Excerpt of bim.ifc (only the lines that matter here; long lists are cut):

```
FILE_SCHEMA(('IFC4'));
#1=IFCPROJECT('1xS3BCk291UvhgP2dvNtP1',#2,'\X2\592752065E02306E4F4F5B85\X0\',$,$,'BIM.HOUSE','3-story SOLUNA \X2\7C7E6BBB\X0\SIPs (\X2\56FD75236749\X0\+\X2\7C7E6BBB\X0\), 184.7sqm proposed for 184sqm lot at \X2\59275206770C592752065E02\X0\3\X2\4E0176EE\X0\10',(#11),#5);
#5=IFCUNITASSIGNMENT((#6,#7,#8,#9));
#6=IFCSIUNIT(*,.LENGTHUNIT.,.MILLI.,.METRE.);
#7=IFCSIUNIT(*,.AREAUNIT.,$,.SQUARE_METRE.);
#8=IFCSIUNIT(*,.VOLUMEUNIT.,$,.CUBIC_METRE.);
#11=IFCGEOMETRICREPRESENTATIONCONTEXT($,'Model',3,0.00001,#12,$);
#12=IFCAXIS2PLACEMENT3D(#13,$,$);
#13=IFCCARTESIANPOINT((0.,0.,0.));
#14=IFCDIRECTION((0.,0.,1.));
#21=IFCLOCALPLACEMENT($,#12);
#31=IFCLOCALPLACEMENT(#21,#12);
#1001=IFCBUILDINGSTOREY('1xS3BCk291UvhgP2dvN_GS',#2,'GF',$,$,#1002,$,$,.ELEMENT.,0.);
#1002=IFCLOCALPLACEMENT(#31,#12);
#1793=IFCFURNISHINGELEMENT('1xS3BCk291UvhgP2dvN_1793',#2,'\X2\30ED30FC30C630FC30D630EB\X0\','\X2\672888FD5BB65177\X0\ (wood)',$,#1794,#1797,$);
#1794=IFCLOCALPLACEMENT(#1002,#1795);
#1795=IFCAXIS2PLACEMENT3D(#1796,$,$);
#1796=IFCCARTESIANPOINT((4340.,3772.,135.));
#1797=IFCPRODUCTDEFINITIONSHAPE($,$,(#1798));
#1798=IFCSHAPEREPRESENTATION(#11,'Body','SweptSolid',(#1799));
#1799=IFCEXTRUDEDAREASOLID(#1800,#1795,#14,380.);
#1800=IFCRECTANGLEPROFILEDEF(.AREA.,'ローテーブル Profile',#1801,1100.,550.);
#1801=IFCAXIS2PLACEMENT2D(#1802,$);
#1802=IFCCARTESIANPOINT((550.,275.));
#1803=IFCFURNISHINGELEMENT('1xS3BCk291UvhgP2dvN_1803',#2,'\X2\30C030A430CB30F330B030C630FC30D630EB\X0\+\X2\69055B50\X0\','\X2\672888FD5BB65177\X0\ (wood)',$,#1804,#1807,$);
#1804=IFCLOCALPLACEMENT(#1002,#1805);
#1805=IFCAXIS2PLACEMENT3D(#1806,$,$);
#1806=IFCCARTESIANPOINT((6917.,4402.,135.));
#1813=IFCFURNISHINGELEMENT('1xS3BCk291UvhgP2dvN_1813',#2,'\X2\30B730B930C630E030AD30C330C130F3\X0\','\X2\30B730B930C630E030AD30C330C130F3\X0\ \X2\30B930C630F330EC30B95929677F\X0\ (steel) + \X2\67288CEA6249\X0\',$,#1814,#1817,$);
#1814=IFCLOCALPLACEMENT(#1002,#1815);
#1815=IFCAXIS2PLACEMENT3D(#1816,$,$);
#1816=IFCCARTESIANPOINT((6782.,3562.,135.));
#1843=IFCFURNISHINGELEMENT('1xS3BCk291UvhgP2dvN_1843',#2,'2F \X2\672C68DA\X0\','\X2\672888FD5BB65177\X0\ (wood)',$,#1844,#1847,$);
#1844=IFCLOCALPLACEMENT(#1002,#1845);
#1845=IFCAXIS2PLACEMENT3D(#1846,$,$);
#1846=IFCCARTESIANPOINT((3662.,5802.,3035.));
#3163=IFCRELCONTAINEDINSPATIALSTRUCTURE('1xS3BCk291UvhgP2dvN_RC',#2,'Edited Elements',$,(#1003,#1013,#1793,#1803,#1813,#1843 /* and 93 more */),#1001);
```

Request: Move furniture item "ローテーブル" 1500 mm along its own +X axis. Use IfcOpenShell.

```python
import ifcopenshell
import ifcopenshell.api.geometry
import ifcopenshell.util.placement
import ifcopenshell.util.unit

model = ifcopenshell.open("bim.ifc")
unit_scale = ifcopenshell.util.unit.calculate_unit_scale(model)

item = model.by_guid("1xS3BCk291UvhgP2dvN_1793")
matrix = ifcopenshell.util.placement.get_local_placement(item.ObjectPlacement)
matrix[:3, 3] += matrix[:3, 0] * 1.5 / unit_scale
ifcopenshell.api.geometry.edit_object_placement(model, product=item, matrix=matrix, is_si=False)

print(ifcopenshell.util.placement.get_local_placement(item.ObjectPlacement).round(3) + 0.0)

model.write("bim_rev.ifc")
```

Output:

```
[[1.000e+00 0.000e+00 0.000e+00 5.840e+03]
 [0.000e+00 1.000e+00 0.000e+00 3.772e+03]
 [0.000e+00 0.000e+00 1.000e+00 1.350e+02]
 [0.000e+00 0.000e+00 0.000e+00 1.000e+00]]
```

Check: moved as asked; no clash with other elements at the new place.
